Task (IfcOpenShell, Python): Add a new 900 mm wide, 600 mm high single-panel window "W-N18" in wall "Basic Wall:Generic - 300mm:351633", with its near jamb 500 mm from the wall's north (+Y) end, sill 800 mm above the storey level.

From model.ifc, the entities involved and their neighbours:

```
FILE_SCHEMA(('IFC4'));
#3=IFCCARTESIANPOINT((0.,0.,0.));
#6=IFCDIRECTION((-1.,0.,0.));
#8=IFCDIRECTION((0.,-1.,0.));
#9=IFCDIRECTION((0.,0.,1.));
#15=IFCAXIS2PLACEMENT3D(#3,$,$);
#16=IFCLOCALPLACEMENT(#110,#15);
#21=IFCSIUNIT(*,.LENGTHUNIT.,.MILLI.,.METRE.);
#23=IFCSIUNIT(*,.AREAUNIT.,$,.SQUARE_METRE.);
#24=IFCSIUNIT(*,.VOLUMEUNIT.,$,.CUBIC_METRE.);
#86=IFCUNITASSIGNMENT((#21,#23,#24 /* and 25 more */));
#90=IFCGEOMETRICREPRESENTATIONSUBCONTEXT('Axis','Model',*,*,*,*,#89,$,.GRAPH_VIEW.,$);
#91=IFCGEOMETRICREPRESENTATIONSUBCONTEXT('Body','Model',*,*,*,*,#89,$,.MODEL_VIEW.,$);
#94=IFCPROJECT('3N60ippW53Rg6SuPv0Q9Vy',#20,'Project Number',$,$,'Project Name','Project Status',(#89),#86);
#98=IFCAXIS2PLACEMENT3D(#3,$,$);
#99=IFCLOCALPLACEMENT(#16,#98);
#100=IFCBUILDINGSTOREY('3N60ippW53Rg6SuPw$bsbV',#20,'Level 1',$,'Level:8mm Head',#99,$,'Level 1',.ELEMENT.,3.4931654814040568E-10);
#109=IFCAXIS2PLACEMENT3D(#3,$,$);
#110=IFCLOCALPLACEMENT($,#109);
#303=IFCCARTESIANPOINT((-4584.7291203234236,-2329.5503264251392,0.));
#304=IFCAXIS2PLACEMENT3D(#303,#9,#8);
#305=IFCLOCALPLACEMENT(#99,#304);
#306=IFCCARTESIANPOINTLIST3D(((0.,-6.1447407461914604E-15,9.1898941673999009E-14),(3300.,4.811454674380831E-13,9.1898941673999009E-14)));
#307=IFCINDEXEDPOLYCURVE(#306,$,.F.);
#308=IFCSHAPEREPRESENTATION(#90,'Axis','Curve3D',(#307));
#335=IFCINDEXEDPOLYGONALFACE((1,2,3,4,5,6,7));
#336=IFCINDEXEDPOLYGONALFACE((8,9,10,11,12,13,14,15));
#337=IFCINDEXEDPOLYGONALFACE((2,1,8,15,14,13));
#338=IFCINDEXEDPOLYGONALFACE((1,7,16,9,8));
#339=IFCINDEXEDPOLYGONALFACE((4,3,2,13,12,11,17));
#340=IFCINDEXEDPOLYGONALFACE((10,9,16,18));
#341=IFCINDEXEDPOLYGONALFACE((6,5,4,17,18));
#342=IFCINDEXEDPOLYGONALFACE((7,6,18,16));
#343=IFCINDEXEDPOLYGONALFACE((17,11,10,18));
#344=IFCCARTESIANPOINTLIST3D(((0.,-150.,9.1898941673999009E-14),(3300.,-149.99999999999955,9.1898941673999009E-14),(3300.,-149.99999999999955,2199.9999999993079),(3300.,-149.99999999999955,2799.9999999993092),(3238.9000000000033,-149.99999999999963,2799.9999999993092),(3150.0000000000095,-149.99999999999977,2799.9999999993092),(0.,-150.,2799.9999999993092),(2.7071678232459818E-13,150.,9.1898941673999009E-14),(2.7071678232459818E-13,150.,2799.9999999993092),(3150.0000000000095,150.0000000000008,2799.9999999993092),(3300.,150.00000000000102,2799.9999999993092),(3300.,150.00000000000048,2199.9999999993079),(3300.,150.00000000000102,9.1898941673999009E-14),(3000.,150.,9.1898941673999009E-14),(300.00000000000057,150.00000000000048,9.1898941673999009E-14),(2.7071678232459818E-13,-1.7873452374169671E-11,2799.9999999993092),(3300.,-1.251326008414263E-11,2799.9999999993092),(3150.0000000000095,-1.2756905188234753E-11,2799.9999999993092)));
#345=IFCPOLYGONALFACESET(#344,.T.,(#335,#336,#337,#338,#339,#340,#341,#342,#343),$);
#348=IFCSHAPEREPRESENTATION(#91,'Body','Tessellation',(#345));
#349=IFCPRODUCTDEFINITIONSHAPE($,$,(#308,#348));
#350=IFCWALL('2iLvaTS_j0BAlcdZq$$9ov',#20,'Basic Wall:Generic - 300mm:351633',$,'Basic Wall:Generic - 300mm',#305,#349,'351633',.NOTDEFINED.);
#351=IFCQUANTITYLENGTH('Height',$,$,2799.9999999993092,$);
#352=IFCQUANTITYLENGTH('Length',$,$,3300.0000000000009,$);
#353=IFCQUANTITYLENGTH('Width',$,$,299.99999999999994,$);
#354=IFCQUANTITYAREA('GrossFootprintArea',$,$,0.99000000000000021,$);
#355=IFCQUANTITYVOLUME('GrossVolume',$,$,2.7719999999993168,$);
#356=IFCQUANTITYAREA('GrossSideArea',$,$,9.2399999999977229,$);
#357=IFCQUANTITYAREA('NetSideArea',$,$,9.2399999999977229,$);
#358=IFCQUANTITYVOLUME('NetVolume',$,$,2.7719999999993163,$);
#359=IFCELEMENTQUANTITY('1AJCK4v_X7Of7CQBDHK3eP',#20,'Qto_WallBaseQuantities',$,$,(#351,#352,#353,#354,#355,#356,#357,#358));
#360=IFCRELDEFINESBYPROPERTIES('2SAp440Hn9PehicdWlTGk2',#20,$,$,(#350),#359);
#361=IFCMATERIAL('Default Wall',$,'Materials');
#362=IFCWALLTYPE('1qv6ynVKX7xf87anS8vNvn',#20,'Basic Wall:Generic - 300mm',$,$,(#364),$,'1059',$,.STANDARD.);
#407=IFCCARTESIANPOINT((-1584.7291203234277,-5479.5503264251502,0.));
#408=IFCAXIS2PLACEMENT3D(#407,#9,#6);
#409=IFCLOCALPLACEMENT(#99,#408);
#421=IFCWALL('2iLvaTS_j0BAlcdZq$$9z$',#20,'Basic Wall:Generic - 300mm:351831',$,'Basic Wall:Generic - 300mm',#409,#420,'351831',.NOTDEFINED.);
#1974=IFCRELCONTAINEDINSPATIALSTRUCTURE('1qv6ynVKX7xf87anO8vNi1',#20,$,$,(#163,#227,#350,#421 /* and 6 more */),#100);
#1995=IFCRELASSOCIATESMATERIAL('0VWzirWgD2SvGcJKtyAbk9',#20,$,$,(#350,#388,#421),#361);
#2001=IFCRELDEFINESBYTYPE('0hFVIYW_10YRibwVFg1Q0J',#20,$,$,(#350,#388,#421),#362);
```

```python
import numpy as np
import ifcopenshell
import ifcopenshell.api.feature
import ifcopenshell.api.geometry
import ifcopenshell.api.pset
import ifcopenshell.api.root
import ifcopenshell.api.spatial
import ifcopenshell.geom
import ifcopenshell.util.element
import ifcopenshell.util.placement
import ifcopenshell.util.representation
import ifcopenshell.util.shape
import ifcopenshell.util.unit

model = ifcopenshell.open("model.ifc")
unit_scale = ifcopenshell.util.unit.calculate_unit_scale(model)
area_scale = ifcopenshell.util.unit.calculate_unit_scale(model, "AREAUNIT")
volume_scale = ifcopenshell.util.unit.calculate_unit_scale(model, "VOLUMEUNIT")
settings = ifcopenshell.geom.settings()


def volume(element):
    """Net volume in cubic metres, openings subtracted."""
    shape = ifcopenshell.geom.create_shape(settings, element)
    return ifcopenshell.util.shape.get_volume(shape.geometry)


wall = model.by_guid("2iLvaTS_j0BAlcdZq$$9ov")
storey = ifcopenshell.util.element.get_container(wall, ifc_class="IfcBuildingStorey")
context = ifcopenshell.util.representation.get_context(model, "Model", "Body", "MODEL_VIEW")
before = volume(wall)

width, height, from_end, sill = 0.9, 0.6, 0.5, 0.8  # metres

# The wall runs along its own X axis, and the end named is its -X end.
wall_shape = ifcopenshell.geom.create_shape(settings, wall)
x, y, z = ifcopenshell.util.shape.get_vertices(wall_shape.geometry).T
start = x.min() + from_end
face, thickness = float(y.min()), float(y.max() - y.min())
wall_matrix = ifcopenshell.util.placement.get_local_placement(wall.ObjectPlacement)
level = ifcopenshell.util.placement.get_local_placement(storey.ObjectPlacement)[2, 3]


def in_wall(x, y):
    """Placement at x, y metres in the wall's axes, at sill height."""
    matrix = wall_matrix.copy()
    matrix[:, 3] = wall_matrix @ np.array([x / unit_scale, y / unit_scale, 0.0, 1.0])
    matrix[2, 3] = level + sill / unit_scale
    return matrix


# Opening: a box that overshoots both wall faces by 50 mm.
opening = ifcopenshell.api.root.create_entity(model, ifc_class="IfcOpeningElement", predefined_type="OPENING")
box = ifcopenshell.api.geometry.add_wall_representation(
    model, context=context, length=width, height=height, thickness=thickness + 0.1
)
ifcopenshell.api.geometry.assign_representation(model, product=opening, representation=box)
ifcopenshell.api.geometry.edit_object_placement(model, product=opening, matrix=in_wall(start, face - 0.05), is_si=False)
ifcopenshell.api.feature.add_feature(model, feature=opening, element=wall)

window = ifcopenshell.api.root.create_entity(model, ifc_class="IfcWindow", name="W-N18", predefined_type="WINDOW")
window.OverallWidth, window.OverallHeight = width / unit_scale, height / unit_scale
window.PartitioningType = "SINGLE_PANEL"
body = ifcopenshell.api.geometry.add_window_representation(
    model,
    context=context,
    overall_width=window.OverallWidth,
    overall_height=window.OverallHeight,
    partition_type="SINGLE_PANEL",
)
ifcopenshell.api.geometry.assign_representation(model, product=window, representation=body)
ifcopenshell.api.spatial.assign_container(model, products=[window], relating_structure=storey)
ifcopenshell.api.feature.add_filling(model, opening=opening, element=window)

# Centre the window in the wall's thickness.
ifcopenshell.api.geometry.edit_object_placement(model, product=window, matrix=in_wall(start, face), is_si=False)
window_shape = ifcopenshell.geom.create_shape(settings, window)
depth = ifcopenshell.util.shape.get_vertices(window_shape.geometry)[:, 1]
offset = face + thickness / 2 - (depth.min() + depth.max()) / 2
ifcopenshell.api.geometry.edit_object_placement(model, product=window, matrix=in_wall(start, offset), is_si=False)

after = volume(wall)

# Update the wall's stored quantities.
qto = model.by_id(ifcopenshell.util.element.get_pset(wall, "Qto_WallBaseQuantities", should_inherit=False)["id"])
ifcopenshell.api.pset.edit_qto(model, qto=qto, properties={
    "NetSideArea": after / thickness / area_scale,
    "NetVolume": after / volume_scale,
})

print(f"wall volume {before:.3f} -> {after:.3f} m3")

model.write("model_rev.ifc")
```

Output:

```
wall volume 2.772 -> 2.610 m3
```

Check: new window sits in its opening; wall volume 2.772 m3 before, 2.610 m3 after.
